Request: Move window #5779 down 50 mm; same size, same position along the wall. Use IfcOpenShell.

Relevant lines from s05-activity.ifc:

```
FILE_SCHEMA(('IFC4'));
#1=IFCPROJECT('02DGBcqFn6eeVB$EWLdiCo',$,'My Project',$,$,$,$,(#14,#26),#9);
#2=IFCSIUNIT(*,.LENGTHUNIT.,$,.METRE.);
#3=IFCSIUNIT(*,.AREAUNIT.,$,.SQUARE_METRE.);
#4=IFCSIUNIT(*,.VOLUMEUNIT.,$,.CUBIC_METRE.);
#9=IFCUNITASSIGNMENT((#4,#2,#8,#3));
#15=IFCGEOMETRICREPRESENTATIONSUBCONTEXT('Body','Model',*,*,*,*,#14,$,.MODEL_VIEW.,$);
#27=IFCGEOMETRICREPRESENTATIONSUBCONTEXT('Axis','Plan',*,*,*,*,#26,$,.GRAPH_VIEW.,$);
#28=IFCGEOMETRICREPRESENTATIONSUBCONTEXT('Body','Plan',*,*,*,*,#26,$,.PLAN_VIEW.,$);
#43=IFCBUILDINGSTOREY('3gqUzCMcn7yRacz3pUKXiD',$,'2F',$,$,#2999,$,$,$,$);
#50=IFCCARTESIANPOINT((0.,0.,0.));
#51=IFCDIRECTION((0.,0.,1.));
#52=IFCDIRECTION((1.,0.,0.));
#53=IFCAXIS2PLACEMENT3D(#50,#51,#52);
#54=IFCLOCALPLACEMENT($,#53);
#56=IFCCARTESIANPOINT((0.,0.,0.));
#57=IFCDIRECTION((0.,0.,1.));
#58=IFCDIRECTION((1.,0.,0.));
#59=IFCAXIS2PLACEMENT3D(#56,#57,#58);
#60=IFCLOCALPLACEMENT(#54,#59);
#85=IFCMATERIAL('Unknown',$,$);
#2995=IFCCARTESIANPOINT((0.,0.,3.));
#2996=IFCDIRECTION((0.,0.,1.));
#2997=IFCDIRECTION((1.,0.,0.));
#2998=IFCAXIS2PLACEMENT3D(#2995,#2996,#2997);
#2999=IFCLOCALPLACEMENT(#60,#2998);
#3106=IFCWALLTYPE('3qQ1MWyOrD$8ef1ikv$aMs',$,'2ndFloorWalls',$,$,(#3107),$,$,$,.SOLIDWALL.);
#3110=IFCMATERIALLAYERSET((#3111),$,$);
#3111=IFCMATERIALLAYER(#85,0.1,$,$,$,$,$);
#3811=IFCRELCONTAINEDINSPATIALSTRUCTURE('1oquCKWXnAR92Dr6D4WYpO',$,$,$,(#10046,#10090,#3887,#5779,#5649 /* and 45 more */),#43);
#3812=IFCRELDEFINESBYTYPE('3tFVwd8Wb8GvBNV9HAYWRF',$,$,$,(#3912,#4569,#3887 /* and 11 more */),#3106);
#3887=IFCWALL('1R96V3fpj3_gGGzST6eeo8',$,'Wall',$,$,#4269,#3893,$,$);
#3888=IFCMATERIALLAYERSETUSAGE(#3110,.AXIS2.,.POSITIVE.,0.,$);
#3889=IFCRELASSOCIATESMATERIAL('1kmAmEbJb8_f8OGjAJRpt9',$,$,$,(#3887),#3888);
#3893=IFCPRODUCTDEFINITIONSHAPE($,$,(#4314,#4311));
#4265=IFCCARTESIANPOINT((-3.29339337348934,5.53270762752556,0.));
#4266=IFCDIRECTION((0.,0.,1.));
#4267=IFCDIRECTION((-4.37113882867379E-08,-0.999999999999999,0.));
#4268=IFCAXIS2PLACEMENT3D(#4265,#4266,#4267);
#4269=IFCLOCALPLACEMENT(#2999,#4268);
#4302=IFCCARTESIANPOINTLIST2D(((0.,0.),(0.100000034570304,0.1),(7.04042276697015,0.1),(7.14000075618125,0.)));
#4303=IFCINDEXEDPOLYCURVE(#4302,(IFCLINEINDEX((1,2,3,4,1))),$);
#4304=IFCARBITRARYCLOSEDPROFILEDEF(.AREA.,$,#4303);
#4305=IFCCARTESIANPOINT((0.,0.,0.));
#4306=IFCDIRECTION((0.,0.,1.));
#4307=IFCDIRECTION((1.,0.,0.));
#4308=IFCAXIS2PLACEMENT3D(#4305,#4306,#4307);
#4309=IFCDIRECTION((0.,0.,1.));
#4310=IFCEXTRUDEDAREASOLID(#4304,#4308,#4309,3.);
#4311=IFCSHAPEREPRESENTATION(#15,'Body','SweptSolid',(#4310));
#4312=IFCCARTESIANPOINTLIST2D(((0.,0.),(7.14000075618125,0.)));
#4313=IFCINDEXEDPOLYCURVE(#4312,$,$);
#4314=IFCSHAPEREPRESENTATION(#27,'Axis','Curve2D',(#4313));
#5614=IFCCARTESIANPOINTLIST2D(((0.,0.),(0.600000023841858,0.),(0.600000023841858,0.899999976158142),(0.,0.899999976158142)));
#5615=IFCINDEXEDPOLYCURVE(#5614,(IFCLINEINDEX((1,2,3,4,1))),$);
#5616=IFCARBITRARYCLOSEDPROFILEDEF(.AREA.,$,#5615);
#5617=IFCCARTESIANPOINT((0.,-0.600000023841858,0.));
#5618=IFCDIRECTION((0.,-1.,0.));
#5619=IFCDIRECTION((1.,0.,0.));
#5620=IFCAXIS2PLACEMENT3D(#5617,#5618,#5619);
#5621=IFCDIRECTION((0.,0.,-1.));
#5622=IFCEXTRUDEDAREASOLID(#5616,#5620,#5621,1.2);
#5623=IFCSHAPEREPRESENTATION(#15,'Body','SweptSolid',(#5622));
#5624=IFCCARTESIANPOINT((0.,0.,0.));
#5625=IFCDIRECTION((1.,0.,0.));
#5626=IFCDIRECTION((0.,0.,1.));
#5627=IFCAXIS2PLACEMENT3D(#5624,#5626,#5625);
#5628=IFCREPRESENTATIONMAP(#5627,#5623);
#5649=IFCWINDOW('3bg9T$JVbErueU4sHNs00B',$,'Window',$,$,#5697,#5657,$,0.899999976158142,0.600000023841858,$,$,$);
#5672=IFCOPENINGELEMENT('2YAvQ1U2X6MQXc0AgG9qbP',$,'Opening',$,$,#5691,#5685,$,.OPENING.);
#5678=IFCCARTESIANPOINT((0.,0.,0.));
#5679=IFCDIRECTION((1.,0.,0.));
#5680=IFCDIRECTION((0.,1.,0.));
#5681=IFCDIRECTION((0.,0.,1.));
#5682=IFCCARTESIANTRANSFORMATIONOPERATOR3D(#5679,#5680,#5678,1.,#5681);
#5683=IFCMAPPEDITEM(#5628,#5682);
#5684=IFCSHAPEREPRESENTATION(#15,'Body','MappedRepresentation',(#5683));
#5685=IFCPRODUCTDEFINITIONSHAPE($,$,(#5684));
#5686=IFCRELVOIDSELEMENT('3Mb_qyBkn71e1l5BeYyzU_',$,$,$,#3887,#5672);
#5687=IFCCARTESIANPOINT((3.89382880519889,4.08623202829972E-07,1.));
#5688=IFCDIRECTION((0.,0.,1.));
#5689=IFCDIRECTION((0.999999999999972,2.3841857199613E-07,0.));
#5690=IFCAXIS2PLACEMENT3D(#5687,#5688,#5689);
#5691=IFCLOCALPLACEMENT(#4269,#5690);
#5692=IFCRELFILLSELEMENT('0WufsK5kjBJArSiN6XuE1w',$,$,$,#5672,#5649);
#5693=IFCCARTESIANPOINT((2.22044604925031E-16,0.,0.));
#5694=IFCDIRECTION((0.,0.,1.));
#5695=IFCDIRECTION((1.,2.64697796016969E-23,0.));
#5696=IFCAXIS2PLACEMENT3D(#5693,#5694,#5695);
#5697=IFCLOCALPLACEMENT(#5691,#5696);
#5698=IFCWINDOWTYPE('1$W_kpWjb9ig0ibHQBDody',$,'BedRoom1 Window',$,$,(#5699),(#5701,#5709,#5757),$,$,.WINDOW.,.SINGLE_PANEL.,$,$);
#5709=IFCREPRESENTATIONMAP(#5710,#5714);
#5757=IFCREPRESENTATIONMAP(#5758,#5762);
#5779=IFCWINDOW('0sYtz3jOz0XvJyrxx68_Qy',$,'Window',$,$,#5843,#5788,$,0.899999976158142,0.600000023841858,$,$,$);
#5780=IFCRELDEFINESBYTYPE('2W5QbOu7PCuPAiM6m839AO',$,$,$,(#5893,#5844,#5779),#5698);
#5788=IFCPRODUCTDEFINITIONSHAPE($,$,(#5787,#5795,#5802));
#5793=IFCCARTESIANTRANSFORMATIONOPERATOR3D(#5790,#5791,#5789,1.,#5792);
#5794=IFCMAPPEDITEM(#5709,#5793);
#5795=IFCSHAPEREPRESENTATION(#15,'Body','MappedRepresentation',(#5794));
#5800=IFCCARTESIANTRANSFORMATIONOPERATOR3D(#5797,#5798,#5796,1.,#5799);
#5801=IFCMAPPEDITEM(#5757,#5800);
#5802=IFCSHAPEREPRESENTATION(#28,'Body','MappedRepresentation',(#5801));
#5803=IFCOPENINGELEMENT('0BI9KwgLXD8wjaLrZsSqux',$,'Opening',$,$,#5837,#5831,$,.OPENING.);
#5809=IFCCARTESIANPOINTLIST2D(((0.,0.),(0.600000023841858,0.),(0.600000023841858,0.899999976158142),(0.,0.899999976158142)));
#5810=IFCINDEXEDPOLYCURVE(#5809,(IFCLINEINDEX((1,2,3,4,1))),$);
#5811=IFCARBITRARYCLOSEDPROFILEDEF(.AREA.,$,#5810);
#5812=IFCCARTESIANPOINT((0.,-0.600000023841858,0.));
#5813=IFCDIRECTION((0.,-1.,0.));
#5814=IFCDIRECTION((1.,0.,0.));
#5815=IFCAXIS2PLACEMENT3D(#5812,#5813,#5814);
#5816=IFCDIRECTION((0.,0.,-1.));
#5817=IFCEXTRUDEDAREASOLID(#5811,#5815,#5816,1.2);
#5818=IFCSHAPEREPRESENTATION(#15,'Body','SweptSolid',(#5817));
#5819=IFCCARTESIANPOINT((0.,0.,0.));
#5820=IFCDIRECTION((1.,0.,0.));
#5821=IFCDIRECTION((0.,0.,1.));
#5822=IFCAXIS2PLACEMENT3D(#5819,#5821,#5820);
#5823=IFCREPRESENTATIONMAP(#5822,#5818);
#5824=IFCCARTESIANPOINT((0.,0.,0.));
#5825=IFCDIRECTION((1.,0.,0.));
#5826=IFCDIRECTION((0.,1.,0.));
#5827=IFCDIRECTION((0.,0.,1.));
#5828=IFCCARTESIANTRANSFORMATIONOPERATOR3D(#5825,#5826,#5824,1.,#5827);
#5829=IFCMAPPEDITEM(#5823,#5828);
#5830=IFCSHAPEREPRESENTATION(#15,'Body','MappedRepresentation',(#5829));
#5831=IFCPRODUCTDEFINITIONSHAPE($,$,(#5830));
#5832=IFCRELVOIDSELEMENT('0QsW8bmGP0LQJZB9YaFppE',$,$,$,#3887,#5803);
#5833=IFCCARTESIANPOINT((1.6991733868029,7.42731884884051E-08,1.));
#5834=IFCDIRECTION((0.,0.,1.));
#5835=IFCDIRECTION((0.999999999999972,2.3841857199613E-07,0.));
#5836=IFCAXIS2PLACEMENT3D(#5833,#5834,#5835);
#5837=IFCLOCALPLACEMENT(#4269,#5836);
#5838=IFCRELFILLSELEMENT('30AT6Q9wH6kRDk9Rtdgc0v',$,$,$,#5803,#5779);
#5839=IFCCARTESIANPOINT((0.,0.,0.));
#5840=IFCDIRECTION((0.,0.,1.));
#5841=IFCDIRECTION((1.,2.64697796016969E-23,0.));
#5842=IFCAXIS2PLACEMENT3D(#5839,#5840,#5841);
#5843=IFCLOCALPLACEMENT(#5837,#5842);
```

```python
import numpy as np
import ifcopenshell
import ifcopenshell.api.geometry
import ifcopenshell.util.placement
import ifcopenshell.util.unit

model = ifcopenshell.open("s05-activity.ifc")
unit_scale = ifcopenshell.util.unit.calculate_unit_scale(model)

window = model.by_id(5779)
opening = window.FillsVoids[0].RelatingOpeningElement
dz = -0.05 / unit_scale

shift = np.array([0.0, 0.0, dz])
# The window is placed relative to its opening, so it follows when the opening moves.
matrix = ifcopenshell.util.placement.get_local_placement(opening.ObjectPlacement)
matrix[:3, 3] += shift
ifcopenshell.api.geometry.edit_object_placement(
    model, product=opening, matrix=matrix, is_si=False, should_transform_children=True
)

print(f"moved by {dz * unit_scale:+.3f} m")

model.write("s05-activity_rev.ifc")
```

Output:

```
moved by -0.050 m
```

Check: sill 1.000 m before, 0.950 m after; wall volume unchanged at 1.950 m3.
